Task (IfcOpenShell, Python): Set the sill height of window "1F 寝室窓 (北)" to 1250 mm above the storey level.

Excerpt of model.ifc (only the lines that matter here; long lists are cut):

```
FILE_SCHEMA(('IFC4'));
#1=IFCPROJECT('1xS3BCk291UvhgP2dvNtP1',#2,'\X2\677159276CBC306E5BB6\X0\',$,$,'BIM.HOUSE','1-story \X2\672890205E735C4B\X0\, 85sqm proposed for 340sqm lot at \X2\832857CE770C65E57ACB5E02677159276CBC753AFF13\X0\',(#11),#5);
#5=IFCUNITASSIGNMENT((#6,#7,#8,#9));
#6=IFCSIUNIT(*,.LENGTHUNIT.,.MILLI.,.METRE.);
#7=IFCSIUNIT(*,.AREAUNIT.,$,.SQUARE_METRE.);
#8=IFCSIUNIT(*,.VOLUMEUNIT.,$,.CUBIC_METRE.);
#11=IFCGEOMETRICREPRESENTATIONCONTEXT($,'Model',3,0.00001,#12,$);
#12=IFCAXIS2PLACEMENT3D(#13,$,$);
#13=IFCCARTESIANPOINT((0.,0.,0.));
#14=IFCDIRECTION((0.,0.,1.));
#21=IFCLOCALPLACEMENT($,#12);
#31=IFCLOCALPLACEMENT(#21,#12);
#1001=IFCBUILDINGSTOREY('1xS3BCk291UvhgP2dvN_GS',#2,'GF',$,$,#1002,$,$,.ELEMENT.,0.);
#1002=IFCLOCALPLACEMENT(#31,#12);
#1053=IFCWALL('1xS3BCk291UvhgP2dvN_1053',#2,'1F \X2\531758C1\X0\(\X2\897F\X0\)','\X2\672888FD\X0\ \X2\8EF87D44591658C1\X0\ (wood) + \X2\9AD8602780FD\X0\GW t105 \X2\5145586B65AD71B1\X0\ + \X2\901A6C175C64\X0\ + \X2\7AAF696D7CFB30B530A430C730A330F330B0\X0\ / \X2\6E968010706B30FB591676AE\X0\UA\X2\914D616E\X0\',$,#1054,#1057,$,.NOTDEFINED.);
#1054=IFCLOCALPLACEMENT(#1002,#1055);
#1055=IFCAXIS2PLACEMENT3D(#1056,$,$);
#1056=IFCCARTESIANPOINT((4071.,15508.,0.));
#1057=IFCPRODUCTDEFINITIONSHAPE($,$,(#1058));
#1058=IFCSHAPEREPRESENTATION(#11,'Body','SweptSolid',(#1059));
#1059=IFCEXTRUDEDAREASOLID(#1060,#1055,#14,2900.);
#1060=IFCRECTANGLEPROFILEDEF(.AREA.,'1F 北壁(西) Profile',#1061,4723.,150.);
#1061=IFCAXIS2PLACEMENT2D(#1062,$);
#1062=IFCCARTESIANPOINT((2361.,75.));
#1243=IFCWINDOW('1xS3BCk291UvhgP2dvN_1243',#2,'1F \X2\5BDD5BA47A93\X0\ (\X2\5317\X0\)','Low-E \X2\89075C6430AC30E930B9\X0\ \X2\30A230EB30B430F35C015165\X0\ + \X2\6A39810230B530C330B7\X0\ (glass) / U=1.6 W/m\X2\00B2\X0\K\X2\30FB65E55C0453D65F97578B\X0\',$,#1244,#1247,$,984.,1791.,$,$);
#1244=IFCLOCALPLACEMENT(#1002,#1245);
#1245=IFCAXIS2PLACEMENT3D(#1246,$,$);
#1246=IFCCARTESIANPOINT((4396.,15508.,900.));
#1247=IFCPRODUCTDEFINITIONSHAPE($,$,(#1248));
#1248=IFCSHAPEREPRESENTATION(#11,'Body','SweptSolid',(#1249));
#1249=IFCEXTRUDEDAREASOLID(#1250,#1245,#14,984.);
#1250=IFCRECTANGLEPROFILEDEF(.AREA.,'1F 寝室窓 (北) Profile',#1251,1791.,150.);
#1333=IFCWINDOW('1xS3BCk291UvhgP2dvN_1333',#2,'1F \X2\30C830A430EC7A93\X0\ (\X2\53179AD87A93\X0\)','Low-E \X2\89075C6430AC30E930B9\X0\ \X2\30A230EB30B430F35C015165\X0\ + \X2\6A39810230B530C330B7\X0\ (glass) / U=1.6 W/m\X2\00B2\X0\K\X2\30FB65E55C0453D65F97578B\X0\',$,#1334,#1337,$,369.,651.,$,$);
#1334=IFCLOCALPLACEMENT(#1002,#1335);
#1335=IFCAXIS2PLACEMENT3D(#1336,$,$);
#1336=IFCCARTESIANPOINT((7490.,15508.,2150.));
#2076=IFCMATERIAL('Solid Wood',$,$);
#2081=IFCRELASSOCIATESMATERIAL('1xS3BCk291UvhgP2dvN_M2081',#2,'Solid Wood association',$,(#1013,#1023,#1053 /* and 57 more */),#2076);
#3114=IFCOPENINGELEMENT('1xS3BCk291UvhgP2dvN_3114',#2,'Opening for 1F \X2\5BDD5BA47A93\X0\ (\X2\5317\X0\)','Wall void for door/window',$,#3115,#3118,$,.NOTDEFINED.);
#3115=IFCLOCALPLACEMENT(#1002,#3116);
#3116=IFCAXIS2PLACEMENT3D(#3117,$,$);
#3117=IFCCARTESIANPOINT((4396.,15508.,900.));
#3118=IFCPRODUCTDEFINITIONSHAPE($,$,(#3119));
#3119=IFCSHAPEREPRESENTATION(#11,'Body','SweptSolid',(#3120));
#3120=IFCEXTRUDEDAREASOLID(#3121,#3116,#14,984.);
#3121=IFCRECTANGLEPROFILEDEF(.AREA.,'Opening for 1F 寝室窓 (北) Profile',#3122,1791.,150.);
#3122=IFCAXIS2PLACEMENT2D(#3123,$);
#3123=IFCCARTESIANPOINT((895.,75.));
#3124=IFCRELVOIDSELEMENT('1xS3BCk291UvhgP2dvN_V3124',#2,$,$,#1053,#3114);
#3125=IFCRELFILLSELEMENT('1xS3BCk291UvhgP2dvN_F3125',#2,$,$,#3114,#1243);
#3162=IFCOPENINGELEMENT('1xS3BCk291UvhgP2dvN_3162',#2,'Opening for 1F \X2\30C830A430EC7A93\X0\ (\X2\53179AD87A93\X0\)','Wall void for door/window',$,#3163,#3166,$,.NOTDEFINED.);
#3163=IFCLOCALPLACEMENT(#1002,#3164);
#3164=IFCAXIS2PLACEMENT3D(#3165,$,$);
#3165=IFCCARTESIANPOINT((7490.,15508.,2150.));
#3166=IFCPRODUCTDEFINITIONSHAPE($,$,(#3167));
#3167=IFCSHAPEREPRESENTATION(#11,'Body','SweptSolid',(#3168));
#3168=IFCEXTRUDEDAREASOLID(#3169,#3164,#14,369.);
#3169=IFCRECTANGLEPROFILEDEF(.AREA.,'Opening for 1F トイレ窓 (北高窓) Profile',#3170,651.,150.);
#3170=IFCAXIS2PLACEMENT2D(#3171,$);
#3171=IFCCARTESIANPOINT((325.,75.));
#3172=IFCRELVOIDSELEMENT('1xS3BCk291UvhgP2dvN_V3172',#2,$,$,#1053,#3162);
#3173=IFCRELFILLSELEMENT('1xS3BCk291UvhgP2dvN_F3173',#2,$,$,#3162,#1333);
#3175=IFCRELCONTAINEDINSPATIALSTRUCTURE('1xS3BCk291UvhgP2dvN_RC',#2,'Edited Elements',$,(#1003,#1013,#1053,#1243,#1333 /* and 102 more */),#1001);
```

```python
import numpy as np
import ifcopenshell
import ifcopenshell.api.geometry
import ifcopenshell.geom
import ifcopenshell.util.element
import ifcopenshell.util.placement
import ifcopenshell.util.shape
import ifcopenshell.util.unit

model = ifcopenshell.open("model.ifc")
unit_scale = ifcopenshell.util.unit.calculate_unit_scale(model)

window = model.by_id(1243)
opening = window.FillsVoids[0].RelatingOpeningElement
storey = ifcopenshell.util.element.get_container(window, ifc_class="IfcBuildingStorey")
level = ifcopenshell.util.placement.get_local_placement(storey.ObjectPlacement)[2, 3]

# The opening's origin need not be at the sill, so measure its lowest point.
shape = ifcopenshell.geom.create_shape(ifcopenshell.geom.settings(), opening)
bottom = ifcopenshell.util.shape.get_shape_bottom_elevation(shape, shape.geometry) / unit_scale
dz = level + 1.25 / unit_scale - bottom

shift = np.array([0.0, 0.0, dz])
# The window is not placed relative to its opening, so move both.
for product in (opening, window):
    matrix = ifcopenshell.util.placement.get_local_placement(product.ObjectPlacement)
    matrix[:3, 3] += shift
    ifcopenshell.api.geometry.edit_object_placement(model, product=product, matrix=matrix, is_si=False)

print(f"moved by {dz * unit_scale:+.3f} m")

model.write("model_v2.ifc")
```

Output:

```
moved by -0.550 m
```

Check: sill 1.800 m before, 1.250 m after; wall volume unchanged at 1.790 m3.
